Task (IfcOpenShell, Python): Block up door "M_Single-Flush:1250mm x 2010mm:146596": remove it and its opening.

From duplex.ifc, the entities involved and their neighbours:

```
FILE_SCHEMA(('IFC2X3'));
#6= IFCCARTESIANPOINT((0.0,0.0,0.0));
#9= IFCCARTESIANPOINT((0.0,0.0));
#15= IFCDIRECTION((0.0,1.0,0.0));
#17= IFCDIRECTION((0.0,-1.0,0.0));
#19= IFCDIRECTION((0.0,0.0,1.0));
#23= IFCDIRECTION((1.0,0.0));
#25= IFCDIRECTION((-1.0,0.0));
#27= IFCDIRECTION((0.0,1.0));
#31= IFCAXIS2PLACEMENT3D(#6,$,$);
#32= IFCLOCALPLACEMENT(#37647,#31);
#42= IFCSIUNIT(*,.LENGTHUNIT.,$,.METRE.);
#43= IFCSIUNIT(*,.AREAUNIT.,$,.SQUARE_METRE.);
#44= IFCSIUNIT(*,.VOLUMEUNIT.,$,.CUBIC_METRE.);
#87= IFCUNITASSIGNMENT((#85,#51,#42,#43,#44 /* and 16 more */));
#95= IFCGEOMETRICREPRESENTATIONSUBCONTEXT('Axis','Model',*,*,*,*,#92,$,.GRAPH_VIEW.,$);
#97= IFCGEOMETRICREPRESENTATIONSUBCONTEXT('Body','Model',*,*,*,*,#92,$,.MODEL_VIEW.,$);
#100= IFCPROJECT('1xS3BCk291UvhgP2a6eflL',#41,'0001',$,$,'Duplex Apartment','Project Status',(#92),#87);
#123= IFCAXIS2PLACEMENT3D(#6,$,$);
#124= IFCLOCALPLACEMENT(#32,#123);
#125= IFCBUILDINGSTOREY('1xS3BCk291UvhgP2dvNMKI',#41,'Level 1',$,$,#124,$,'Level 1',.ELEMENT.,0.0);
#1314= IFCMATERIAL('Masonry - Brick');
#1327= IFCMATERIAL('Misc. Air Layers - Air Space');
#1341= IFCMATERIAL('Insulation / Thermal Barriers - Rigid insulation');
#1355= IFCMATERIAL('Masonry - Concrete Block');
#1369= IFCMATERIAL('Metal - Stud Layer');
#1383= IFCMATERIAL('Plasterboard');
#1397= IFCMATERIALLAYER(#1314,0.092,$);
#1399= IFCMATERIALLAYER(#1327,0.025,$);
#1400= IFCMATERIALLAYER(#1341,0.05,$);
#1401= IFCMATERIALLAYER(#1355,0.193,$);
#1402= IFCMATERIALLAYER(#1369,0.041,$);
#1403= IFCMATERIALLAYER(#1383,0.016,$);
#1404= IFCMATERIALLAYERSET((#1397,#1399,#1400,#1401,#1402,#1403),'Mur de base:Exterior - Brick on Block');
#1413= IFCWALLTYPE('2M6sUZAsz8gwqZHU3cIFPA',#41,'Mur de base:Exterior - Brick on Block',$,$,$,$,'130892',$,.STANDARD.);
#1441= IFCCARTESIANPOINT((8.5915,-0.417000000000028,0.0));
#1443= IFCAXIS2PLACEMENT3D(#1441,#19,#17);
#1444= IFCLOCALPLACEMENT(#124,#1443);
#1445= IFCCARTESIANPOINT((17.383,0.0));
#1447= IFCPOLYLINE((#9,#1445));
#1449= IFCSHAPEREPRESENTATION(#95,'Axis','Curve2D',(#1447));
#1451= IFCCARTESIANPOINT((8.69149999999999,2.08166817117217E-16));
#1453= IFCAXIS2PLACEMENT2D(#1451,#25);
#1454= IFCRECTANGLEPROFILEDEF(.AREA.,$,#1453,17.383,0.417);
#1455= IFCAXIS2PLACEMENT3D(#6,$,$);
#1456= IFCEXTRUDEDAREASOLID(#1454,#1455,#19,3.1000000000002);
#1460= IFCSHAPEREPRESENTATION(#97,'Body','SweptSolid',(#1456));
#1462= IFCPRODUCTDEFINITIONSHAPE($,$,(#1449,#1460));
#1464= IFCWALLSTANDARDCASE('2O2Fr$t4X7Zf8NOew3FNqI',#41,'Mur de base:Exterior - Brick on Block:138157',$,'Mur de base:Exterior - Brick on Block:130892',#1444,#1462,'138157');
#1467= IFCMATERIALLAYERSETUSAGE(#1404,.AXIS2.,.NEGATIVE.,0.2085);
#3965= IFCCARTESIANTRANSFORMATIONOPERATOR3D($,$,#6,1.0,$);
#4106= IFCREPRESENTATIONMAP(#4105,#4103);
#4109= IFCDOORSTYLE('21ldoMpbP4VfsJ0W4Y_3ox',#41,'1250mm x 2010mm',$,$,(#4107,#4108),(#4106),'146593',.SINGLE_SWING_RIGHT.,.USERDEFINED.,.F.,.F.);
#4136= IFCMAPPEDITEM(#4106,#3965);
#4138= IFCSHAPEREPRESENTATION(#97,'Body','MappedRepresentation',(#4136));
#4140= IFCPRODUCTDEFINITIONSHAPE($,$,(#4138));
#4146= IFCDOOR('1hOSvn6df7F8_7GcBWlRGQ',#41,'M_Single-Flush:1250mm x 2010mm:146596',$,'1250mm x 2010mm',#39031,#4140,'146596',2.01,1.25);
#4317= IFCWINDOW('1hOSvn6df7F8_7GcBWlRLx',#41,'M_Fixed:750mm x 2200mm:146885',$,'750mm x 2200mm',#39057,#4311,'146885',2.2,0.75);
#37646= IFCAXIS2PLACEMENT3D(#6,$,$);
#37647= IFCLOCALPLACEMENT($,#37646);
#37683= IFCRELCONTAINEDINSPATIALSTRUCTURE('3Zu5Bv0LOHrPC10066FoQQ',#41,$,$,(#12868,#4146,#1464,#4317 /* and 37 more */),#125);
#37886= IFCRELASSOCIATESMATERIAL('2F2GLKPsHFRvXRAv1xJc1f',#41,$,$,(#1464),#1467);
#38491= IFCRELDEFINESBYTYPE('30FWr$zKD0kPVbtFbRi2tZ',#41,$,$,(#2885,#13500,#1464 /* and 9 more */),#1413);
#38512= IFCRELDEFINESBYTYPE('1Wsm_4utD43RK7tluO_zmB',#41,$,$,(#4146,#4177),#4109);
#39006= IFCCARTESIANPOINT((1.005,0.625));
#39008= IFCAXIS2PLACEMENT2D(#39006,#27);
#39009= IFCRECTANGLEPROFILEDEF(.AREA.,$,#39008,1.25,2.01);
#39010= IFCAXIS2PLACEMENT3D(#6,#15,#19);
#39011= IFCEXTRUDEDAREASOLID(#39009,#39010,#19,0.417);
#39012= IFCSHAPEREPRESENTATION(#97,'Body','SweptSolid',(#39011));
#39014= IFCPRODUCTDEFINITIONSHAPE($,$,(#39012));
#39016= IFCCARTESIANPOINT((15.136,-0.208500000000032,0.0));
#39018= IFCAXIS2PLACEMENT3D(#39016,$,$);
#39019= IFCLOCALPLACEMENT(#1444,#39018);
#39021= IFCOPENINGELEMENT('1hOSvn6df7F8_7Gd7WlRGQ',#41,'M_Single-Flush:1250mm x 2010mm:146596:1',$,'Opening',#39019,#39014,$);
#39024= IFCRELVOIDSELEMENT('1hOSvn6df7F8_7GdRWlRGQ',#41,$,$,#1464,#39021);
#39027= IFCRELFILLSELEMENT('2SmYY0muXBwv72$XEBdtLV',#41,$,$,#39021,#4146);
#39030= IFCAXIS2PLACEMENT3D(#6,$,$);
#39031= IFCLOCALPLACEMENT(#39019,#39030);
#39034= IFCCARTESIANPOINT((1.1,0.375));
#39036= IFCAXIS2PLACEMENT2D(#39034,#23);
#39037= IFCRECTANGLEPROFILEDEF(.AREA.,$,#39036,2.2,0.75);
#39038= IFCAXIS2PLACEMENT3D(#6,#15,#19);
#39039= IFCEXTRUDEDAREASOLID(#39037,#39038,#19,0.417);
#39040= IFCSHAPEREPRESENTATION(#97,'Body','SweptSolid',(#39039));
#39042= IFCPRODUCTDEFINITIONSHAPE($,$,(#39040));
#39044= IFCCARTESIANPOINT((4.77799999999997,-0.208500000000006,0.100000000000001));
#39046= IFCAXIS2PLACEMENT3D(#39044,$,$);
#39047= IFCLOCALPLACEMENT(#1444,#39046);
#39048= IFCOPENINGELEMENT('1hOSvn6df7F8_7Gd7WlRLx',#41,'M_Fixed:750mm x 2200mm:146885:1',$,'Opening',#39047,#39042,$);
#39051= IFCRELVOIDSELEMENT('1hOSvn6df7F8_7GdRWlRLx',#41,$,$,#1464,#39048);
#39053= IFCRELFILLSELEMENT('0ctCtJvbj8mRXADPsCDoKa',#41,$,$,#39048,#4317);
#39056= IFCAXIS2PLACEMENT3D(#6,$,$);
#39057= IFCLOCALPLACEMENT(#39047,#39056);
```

```python
import ifcopenshell
import ifcopenshell.api.feature
import ifcopenshell.api.root
import ifcopenshell.geom
import ifcopenshell.util.shape

model = ifcopenshell.open("duplex.ifc")
settings = ifcopenshell.geom.settings()


def volume(element):
    """Net volume in cubic metres, openings subtracted."""
    shape = ifcopenshell.geom.create_shape(settings, element)
    return ifcopenshell.util.shape.get_volume(shape.geometry)


door = model.by_guid("1hOSvn6df7F8_7GcBWlRGQ")
opening = door.FillsVoids[0].RelatingOpeningElement
wall = opening.VoidsElements[0].RelatingBuildingElement
before = volume(wall)

ifcopenshell.api.root.remove_product(model, product=door)
ifcopenshell.api.feature.remove_feature(model, feature=opening)

after = volume(wall)

print(f"wall volume {before:.3f} -> {after:.3f} m3")

model.write("duplex_updated.ifc")
```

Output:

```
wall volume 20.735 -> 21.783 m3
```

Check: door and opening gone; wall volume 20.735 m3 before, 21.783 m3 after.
